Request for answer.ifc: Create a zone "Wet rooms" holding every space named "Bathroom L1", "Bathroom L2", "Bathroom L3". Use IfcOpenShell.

First a look at what the model holds.

```python
import ifcopenshell

model = ifcopenshell.open("answer.ifc")
print(model.schema)
seen = {}
for space in model.by_type("IfcSpace"):
    seen[space.Name] = seen.get(space.Name, 0) + 1
for name, count in sorted(seen.items(), key=str):
    print(count, "x", name)
print("zones:", [z.Name for z in model.by_type("IfcZone")][:20])
```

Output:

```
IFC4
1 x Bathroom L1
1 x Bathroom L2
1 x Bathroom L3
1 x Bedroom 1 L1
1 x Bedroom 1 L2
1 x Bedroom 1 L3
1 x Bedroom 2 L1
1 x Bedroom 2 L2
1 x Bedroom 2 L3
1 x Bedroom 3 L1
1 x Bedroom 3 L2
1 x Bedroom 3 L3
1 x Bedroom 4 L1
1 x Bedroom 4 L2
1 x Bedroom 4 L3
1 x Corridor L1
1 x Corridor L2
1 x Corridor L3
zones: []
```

```python
import ifcopenshell
import ifcopenshell.api.group
import ifcopenshell.api.root

model = ifcopenshell.open("answer.ifc")

names = {"Bathroom L1", "Bathroom L2", "Bathroom L3"}
spaces = [s for s in model.by_type("IfcSpace") if s.Name in names]

zone = ifcopenshell.api.root.create_entity(model, ifc_class="IfcZone", name="Wet rooms")
ifcopenshell.api.group.assign_group(model, products=spaces, group=zone)
print(len(spaces), "spaces in", zone.Name)

model.write("answer_rev.ifc")
```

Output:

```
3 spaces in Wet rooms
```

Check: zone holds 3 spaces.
